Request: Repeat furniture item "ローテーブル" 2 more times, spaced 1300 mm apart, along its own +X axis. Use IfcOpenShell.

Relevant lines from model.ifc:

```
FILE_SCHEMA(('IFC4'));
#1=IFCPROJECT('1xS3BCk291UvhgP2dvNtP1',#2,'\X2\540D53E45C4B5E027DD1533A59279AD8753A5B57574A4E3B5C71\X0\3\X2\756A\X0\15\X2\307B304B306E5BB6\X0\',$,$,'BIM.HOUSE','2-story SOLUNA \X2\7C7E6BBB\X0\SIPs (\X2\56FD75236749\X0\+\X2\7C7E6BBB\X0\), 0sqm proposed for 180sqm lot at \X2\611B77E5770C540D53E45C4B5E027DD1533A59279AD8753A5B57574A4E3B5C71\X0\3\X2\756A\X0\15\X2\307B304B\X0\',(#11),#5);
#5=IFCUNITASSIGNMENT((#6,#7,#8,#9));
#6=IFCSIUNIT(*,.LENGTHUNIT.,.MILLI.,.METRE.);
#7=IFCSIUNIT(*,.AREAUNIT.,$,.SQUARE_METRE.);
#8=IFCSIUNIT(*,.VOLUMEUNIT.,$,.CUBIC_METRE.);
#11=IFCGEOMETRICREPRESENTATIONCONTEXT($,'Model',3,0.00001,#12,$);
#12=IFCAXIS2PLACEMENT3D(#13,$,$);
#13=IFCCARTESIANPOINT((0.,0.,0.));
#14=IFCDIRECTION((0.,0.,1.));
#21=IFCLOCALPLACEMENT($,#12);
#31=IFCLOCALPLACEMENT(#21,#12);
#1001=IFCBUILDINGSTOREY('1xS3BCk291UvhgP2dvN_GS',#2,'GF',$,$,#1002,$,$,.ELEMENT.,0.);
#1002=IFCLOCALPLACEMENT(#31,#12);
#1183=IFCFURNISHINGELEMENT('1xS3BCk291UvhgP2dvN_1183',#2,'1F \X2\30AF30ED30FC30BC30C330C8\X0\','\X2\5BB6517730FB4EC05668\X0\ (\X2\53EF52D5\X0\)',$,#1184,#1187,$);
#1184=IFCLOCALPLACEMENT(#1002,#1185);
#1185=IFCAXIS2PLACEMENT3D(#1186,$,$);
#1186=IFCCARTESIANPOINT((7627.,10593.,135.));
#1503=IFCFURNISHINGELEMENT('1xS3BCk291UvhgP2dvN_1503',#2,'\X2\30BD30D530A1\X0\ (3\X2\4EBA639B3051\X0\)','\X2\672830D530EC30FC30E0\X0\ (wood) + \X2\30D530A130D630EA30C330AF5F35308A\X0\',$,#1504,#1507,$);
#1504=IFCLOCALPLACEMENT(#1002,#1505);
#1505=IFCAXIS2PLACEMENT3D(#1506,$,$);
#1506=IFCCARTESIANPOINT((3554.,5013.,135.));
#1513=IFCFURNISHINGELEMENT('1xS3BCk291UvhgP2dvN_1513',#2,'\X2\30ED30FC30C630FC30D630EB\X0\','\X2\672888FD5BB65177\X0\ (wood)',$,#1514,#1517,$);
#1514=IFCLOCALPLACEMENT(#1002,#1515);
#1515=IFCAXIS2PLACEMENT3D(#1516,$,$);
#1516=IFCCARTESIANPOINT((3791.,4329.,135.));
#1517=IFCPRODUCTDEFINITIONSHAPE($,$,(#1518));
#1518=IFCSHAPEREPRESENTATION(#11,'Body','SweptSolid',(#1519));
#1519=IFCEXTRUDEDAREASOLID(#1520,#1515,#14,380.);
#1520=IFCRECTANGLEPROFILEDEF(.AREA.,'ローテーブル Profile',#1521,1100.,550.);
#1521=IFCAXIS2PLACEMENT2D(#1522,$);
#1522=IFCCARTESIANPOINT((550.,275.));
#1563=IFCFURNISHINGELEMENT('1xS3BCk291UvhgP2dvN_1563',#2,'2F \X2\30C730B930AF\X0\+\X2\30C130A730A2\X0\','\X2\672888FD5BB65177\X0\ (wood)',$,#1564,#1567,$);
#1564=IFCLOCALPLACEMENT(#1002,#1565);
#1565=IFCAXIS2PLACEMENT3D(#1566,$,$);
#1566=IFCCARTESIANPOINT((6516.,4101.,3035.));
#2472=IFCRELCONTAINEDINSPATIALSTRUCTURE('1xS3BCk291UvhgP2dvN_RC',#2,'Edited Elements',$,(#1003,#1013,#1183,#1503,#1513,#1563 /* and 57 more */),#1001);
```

```python
import ifcopenshell
import ifcopenshell.api.geometry
import ifcopenshell.api.root
import ifcopenshell.util.element
import ifcopenshell.util.placement

model = ifcopenshell.open("model.ifc")


def reuse_history(source, copy):
    """copy_class also copies each property set's owner history, people and application; keep the originals."""
    for rel in copy.IsDefinedBy:
        if rel.is_a("IfcRelDefinesByProperties") and (history := rel.RelatingPropertyDefinition.OwnerHistory):
            rel.RelatingPropertyDefinition.OwnerHistory = source.OwnerHistory
            ifcopenshell.util.element.remove_deep2(model, history)


source = model.by_guid("1xS3BCk291UvhgP2dvN_1513")
base = ifcopenshell.util.placement.get_local_placement(source.ObjectPlacement)
step = base[:3, 0] * 1300.0

for i in range(1, 3):
    copy = ifcopenshell.api.root.copy_class(model, product=source)
    copy.Representation = ifcopenshell.util.element.copy_deep(
        model, source.Representation, exclude=["IfcGeometricRepresentationContext", "IfcRepresentationMap"]
    )
    reuse_history(source, copy)
    matrix = base.copy()
    matrix[:3, 3] += i * step
    print("added at", matrix[:3, 3].round(3) + 0.0)
    ifcopenshell.api.geometry.edit_object_placement(model, product=copy, matrix=matrix, is_si=False)

model.write("model_updated.ifc")
```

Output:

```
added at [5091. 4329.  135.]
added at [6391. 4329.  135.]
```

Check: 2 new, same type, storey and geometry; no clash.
